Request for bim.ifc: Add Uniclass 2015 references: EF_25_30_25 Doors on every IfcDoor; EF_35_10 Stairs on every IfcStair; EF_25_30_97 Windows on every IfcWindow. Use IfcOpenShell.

First a look at what the model holds.

```python
import ifcopenshell

model = ifcopenshell.open("bim.ifc")
print(model.schema)
print("classifications:", [c.Name for c in model.by_type("IfcClassification")])
for ifc_class in ("IfcDoor", "IfcRoof", "IfcStair", "IfcWall", "IfcWindow"):
    print(ifc_class, len(model.by_type(ifc_class)))
```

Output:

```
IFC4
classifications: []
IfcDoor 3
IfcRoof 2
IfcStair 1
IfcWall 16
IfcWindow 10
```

```python
import ifcopenshell
import ifcopenshell.api.classification

model = ifcopenshell.open("bim.ifc")

system = ifcopenshell.api.classification.add_classification(model, classification="Uniclass 2015")

codes = {
    "IfcDoor": ("EF_25_30_25", "Doors"),
    "IfcStair": ("EF_35_10", "Stairs"),
    "IfcWindow": ("EF_25_30_97", "Windows"),
}
for ifc_class, (code, name) in codes.items():
    products = model.by_type(ifc_class)
    ifcopenshell.api.classification.add_reference(
        model, products=products, classification=system, identification=code, name=name
    )
    print(code, len(products))

model.write("bim_edited.ifc")
```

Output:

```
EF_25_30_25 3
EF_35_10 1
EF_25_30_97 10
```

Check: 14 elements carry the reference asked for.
